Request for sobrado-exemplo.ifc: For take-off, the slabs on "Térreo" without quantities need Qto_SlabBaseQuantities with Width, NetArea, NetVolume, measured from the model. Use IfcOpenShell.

First a look at what the model holds.

```python
import ifcopenshell
import ifcopenshell.util.element
import ifcopenshell.util.unit

model = ifcopenshell.open("sobrado-exemplo.ifc")
print(model.schema)
for unit_type in ("LENGTHUNIT", "AREAUNIT", "VOLUMEUNIT"):
    print(unit_type, ifcopenshell.util.unit.calculate_unit_scale(model, unit_type))
storey = next(s for s in model.by_type("IfcBuildingStorey") if s.Name == "Térreo")
slabs = [e for e in ifcopenshell.util.element.get_decomposition(storey) if e.is_a("IfcSlab")]
for e in sorted(slabs, key=lambda e: e.id()):
    print(e.id(), e.is_a(), e.Name, list(ifcopenshell.util.element.get_psets(e, qtos_only=True)), sep=" | ")
```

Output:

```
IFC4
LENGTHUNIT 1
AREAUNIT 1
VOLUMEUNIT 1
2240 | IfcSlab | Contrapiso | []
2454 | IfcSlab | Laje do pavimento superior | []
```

```python
import ifcopenshell
import ifcopenshell.api.pset
import ifcopenshell.geom
import ifcopenshell.util.element
import ifcopenshell.util.shape
import ifcopenshell.util.unit

model = ifcopenshell.open("sobrado-exemplo.ifc")
unit_scale = ifcopenshell.util.unit.calculate_unit_scale(model)
area_scale = ifcopenshell.util.unit.calculate_unit_scale(model, "AREAUNIT")
volume_scale = ifcopenshell.util.unit.calculate_unit_scale(model, "VOLUMEUNIT")
settings = ifcopenshell.geom.settings()

storey = next(s for s in model.by_type("IfcBuildingStorey") if s.Name == "Térreo")
slabs = [e for e in ifcopenshell.util.element.get_decomposition(storey) if e.is_a("IfcSlab")]

for e in sorted(slabs, key=lambda e: e.id()):
    if ifcopenshell.util.element.get_psets(e, qtos_only=True, should_inherit=False):
        continue
    # Geometry comes back in metres, in the element's own axes.
    shape = ifcopenshell.geom.create_shape(settings, e)
    values = {
        "Width": ifcopenshell.util.shape.get_z(shape.geometry) / unit_scale,
        "NetArea": ifcopenshell.util.shape.get_footprint_area(shape.geometry) / area_scale,
        "NetVolume": ifcopenshell.util.shape.get_volume(shape.geometry) / volume_scale,
    }
    qto = ifcopenshell.api.pset.add_qto(model, product=e, name="Qto_SlabBaseQuantities")
    ifcopenshell.api.pset.edit_qto(model, qto=qto, properties=values)
    print(e.id(), {k: round(v, 3) for k, v in values.items()})

model.write("sobrado-exemplo-out.ifc")
```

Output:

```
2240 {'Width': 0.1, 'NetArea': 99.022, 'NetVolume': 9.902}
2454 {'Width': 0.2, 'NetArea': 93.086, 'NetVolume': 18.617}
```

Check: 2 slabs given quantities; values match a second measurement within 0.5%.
